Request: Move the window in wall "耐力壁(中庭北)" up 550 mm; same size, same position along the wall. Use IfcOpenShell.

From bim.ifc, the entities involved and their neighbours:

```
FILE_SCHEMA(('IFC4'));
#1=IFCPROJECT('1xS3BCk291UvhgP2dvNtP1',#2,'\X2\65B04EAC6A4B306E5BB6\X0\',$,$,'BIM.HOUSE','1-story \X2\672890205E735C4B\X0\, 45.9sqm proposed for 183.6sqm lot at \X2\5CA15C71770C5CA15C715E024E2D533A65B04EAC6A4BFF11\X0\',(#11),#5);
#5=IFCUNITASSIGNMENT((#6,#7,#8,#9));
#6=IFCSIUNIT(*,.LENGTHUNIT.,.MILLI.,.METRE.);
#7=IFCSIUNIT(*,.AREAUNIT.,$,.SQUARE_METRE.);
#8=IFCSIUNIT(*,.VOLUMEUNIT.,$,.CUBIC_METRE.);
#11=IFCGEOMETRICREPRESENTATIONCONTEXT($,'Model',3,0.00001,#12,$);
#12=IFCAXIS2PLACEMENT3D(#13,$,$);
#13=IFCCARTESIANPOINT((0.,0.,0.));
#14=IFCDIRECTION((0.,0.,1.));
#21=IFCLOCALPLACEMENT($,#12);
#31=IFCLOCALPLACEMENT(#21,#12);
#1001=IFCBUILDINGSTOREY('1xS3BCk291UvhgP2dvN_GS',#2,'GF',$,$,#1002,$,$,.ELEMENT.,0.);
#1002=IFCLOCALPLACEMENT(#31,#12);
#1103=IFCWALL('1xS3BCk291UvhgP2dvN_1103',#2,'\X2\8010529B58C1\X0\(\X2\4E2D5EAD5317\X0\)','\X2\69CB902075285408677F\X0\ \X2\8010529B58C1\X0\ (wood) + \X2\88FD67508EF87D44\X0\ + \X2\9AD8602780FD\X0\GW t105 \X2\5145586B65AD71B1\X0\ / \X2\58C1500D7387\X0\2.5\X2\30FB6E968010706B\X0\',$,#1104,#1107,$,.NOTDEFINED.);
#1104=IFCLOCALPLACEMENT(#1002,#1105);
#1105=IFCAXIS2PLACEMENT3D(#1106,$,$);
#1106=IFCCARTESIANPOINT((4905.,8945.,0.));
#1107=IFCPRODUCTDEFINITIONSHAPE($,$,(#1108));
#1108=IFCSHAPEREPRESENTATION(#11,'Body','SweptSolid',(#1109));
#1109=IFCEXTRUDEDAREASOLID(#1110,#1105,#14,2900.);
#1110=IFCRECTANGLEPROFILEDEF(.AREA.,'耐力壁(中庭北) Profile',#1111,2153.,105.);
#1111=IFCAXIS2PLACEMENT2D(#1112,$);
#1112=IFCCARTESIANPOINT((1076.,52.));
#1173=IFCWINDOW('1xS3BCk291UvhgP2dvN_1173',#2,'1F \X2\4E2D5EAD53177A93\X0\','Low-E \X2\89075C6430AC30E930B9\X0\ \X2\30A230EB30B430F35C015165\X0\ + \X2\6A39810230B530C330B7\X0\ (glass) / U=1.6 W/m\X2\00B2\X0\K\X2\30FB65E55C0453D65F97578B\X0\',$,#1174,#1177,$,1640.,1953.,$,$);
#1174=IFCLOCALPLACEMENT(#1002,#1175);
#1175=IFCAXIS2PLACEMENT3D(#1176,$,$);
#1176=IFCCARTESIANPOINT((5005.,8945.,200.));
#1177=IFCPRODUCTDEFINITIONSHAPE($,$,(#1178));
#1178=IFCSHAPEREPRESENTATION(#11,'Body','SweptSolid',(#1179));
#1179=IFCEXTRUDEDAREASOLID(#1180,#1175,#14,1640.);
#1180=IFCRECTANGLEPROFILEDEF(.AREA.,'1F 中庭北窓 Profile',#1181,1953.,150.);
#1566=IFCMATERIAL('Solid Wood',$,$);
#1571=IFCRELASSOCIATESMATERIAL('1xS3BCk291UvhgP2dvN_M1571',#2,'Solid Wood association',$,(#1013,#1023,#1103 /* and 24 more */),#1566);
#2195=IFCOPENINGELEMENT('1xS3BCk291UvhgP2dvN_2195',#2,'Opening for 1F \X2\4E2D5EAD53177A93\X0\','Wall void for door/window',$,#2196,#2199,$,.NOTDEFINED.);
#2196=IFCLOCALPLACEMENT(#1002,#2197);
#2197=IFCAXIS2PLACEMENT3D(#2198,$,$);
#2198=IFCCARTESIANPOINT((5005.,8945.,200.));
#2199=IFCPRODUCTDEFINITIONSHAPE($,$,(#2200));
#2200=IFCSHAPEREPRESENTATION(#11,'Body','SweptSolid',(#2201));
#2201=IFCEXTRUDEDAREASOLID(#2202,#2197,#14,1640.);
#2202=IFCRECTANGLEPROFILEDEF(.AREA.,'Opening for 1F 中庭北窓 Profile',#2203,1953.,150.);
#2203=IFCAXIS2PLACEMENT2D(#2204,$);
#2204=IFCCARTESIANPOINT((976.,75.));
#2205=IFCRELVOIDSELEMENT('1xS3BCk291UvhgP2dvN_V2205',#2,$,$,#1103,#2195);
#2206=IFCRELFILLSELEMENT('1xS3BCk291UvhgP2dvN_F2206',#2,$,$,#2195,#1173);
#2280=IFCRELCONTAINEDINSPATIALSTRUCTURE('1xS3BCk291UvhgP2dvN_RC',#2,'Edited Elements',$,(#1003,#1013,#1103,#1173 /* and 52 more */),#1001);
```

```python
import numpy as np
import ifcopenshell
import ifcopenshell.api.geometry
import ifcopenshell.util.placement
import ifcopenshell.util.unit

model = ifcopenshell.open("bim.ifc")
unit_scale = ifcopenshell.util.unit.calculate_unit_scale(model)

window = model.by_id(1173)
opening = window.FillsVoids[0].RelatingOpeningElement
dz = 0.55 / unit_scale

shift = np.array([0.0, 0.0, dz])
# The window is not placed relative to its opening, so move both.
for product in (opening, window):
    matrix = ifcopenshell.util.placement.get_local_placement(product.ObjectPlacement)
    matrix[:3, 3] += shift
    ifcopenshell.api.geometry.edit_object_placement(model, product=product, matrix=matrix, is_si=False)

print(f"moved by {dz * unit_scale:+.3f} m")

model.write("bim_edited.ifc")
```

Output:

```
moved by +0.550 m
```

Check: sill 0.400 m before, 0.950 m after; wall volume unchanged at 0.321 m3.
